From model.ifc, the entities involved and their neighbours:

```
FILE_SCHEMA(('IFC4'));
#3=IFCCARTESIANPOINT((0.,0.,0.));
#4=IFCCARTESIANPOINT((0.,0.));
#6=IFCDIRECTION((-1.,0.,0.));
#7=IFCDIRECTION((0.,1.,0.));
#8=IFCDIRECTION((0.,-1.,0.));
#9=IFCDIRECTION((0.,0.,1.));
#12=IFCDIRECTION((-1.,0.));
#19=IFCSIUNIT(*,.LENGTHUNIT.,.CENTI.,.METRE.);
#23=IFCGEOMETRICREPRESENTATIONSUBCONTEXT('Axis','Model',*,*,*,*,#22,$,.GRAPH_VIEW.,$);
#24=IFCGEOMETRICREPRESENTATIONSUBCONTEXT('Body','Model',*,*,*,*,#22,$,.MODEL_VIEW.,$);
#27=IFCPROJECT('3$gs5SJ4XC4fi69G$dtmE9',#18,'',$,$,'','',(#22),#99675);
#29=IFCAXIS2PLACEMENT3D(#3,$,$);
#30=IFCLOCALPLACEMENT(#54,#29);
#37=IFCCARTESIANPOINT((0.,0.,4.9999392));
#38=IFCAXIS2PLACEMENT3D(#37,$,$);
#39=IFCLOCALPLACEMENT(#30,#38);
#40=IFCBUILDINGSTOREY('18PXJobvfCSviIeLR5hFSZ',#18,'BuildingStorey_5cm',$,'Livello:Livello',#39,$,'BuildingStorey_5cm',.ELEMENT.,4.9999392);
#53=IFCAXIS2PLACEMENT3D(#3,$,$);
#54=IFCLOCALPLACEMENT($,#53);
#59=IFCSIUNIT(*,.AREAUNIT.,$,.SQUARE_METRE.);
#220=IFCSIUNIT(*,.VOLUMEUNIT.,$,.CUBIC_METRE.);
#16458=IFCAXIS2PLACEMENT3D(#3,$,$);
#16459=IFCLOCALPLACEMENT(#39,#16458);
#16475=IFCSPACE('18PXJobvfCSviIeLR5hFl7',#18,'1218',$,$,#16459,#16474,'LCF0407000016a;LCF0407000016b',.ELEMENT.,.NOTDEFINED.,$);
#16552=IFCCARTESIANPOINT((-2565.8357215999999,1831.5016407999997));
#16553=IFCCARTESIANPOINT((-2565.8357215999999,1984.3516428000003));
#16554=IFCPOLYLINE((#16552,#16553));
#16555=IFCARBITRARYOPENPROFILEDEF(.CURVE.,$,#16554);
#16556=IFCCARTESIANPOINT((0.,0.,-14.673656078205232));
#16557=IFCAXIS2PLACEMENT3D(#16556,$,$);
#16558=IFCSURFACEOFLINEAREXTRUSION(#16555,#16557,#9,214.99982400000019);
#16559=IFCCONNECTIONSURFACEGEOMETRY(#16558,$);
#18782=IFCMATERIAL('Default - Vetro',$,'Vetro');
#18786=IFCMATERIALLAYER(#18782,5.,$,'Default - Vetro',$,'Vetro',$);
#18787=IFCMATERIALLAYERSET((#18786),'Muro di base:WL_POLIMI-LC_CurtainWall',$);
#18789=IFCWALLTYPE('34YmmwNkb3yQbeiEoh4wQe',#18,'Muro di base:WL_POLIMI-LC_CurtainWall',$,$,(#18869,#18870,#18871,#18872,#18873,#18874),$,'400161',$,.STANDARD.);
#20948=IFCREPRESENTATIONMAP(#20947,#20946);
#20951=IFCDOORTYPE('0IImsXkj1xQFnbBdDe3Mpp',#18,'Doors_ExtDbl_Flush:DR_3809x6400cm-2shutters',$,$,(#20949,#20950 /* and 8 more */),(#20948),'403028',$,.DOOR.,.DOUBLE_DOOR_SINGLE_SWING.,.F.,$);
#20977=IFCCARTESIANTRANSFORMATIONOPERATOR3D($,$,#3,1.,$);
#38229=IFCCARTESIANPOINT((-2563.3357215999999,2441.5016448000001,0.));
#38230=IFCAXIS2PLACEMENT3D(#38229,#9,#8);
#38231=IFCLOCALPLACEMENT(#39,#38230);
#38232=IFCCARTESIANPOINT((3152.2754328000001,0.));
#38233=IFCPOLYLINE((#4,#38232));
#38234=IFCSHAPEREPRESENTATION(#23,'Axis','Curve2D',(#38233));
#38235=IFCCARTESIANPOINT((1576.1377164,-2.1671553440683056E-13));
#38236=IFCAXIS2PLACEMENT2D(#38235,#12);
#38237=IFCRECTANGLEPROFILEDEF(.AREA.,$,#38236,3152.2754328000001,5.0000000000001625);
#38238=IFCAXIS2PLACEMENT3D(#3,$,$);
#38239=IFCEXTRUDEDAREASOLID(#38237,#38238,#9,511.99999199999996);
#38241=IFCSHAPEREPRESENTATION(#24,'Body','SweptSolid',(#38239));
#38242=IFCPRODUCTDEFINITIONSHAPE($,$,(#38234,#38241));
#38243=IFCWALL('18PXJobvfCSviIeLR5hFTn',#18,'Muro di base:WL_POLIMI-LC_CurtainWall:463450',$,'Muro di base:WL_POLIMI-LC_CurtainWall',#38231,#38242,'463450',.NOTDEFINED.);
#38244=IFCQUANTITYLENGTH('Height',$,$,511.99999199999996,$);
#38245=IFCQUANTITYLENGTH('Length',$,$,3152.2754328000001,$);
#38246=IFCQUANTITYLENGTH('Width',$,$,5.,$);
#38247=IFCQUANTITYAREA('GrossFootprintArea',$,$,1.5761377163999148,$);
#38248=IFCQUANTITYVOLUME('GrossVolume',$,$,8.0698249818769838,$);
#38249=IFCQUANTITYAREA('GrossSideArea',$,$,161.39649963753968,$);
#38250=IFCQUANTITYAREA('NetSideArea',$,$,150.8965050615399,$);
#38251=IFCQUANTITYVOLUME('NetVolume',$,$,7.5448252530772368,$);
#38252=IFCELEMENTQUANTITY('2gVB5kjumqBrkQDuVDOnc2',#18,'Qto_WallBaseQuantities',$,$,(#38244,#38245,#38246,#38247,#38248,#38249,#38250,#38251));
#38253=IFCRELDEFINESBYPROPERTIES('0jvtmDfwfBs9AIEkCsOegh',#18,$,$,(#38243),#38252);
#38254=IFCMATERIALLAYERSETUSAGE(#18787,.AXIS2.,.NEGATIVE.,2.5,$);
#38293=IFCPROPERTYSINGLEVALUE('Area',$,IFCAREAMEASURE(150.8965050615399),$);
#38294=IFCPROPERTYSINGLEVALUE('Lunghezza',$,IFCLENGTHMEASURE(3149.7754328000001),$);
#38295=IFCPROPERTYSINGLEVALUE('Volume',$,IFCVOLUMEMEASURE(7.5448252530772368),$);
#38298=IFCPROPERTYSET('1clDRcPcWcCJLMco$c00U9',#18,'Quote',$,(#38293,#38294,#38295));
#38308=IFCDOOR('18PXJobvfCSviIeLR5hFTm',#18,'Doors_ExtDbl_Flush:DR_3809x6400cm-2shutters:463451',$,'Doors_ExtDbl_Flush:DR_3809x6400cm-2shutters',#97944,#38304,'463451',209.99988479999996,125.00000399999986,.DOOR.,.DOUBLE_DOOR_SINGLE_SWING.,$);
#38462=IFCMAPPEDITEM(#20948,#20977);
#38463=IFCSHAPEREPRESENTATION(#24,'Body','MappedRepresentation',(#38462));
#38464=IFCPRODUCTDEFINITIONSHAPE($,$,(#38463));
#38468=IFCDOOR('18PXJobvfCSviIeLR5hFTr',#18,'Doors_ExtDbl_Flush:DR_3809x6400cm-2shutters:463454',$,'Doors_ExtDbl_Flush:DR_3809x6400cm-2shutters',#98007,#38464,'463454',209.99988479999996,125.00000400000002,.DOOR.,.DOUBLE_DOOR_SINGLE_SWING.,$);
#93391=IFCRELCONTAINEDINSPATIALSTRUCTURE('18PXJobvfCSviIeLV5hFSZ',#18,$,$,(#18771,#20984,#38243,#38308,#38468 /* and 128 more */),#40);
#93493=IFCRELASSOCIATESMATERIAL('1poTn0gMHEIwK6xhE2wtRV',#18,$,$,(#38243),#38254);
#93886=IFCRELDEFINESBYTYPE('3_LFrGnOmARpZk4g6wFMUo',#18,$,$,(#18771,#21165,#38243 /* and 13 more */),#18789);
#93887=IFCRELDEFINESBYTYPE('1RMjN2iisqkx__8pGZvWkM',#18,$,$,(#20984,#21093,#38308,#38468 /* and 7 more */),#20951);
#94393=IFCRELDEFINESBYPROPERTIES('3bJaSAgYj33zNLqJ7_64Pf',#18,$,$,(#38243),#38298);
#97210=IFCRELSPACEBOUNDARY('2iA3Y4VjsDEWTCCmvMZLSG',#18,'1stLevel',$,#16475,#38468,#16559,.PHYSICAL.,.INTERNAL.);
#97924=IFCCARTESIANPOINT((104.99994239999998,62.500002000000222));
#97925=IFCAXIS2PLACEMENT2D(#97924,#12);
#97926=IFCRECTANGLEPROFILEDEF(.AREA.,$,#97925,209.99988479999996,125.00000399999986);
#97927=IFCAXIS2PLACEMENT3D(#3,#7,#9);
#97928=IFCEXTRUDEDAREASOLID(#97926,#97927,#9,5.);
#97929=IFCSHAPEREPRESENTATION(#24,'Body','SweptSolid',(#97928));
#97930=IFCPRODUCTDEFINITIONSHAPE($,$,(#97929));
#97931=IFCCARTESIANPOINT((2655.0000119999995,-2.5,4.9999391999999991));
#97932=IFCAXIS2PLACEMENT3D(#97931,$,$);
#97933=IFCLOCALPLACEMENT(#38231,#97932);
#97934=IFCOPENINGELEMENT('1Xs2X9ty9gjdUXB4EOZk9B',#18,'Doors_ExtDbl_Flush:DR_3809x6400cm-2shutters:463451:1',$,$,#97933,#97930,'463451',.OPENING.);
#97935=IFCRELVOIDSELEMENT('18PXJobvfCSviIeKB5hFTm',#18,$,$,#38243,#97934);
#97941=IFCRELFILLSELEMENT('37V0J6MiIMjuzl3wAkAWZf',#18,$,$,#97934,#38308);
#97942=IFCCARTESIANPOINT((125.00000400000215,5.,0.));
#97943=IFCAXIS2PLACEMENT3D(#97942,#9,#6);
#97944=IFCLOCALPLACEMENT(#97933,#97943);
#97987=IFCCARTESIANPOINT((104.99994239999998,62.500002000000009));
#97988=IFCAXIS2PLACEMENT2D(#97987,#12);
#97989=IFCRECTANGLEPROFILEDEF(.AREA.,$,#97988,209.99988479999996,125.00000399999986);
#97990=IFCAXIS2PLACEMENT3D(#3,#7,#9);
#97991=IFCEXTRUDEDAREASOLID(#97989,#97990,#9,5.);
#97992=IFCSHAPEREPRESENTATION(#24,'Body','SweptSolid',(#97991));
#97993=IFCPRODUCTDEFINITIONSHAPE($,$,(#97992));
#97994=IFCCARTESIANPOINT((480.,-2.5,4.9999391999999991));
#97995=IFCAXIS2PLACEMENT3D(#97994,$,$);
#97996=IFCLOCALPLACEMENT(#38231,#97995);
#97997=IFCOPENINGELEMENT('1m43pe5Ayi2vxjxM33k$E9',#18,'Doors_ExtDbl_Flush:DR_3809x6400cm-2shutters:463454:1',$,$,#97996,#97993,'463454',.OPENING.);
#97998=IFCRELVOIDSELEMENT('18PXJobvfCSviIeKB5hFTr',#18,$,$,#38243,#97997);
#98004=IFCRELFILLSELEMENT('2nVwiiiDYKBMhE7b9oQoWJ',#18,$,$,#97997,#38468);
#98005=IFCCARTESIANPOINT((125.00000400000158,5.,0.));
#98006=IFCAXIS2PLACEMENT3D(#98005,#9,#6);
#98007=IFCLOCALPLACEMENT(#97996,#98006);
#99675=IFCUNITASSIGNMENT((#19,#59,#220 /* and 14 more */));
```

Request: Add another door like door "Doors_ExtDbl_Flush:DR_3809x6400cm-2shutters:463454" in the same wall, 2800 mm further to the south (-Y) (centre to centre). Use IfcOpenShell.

```python
import numpy as np
import ifcopenshell
import ifcopenshell.api.feature
import ifcopenshell.api.geometry
import ifcopenshell.api.pset
import ifcopenshell.api.root
import ifcopenshell.geom
import ifcopenshell.util.element
import ifcopenshell.util.placement
import ifcopenshell.util.shape
import ifcopenshell.util.unit

model = ifcopenshell.open("model.ifc")
unit_scale = ifcopenshell.util.unit.calculate_unit_scale(model)
area_scale = ifcopenshell.util.unit.calculate_unit_scale(model, "AREAUNIT")
volume_scale = ifcopenshell.util.unit.calculate_unit_scale(model, "VOLUMEUNIT")
settings = ifcopenshell.geom.settings()


def volume(element):
    """Net volume in cubic metres, openings subtracted."""
    shape = ifcopenshell.geom.create_shape(settings, element)
    return ifcopenshell.util.shape.get_volume(shape.geometry)


def reuse_history(source, copy):
    """copy_class also copies each property set's owner history, people and application; keep the originals."""
    for rel in copy.IsDefinedBy:
        if rel.is_a("IfcRelDefinesByProperties") and (history := rel.RelatingPropertyDefinition.OwnerHistory):
            rel.RelatingPropertyDefinition.OwnerHistory = source.OwnerHistory
            ifcopenshell.util.element.remove_deep2(model, history)


door = model.by_guid("18PXJobvfCSviIeLR5hFTr")
opening = door.FillsVoids[0].RelatingOpeningElement
wall = opening.VoidsElements[0].RelatingBuildingElement
before = volume(wall)
shift = ifcopenshell.util.placement.get_local_placement(wall.ObjectPlacement)[:3, 0] * 2.8 / unit_scale

# copy_class copies the void relationship, type, container and properties, but no geometry.
new_opening = ifcopenshell.api.root.copy_class(model, product=opening)
new_opening.Representation = ifcopenshell.util.element.copy_deep(
    model, opening.Representation, exclude=["IfcGeometricRepresentationContext", "IfcRepresentationMap"]
)
new_opening.Name = "Doors_ExtDbl_Flush:DR_3809x6400cm-2shutters"
new_opening.Tag = None
reuse_history(opening, new_opening)
new_door = ifcopenshell.api.root.copy_class(model, product=door)
new_door.Representation = ifcopenshell.util.element.copy_deep(
    model, door.Representation, exclude=["IfcGeometricRepresentationContext", "IfcRepresentationMap"]
)
new_door.Name = "Doors_ExtDbl_Flush:DR_3809x6400cm-2shutters"
new_door.Tag = None
reuse_history(door, new_door)
ifcopenshell.api.feature.add_filling(model, opening=new_opening, element=new_door)

for old, new in ((opening, new_opening), (door, new_door)):
    matrix = ifcopenshell.util.placement.get_local_placement(old.ObjectPlacement)
    matrix[:3, 3] += shift
    ifcopenshell.api.geometry.edit_object_placement(model, product=new, matrix=matrix, is_si=False)

# The copied space boundaries still share their surfaces with the original.
for rel in new_door.ProvidesBoundaries:
    if rel.ConnectionGeometry:
        rel.ConnectionGeometry = ifcopenshell.util.element.copy_deep(model, rel.ConnectionGeometry)

# Space boundary surfaces are stored in each space's coordinates; move them too.
for rel in new_door.ProvidesBoundaries:
    if not rel.ConnectionGeometry:
        continue
    surface = rel.ConnectionGeometry.SurfaceOnRelatingElement
    space_matrix = ifcopenshell.util.placement.get_local_placement(rel.RelatingSpace.ObjectPlacement)
    point = np.array(surface.Position.Location.Coordinates) + space_matrix[:3, :3].T @ shift
    surface.Position = model.createIfcAxis2Placement3D(
        model.createIfcCartesianPoint(point.tolist()), surface.Position.Axis, surface.Position.RefDirection
    )

after = volume(wall)
thickness = 0.05  # wall thickness in metres

# Update the wall's stored quantities.
qto = model.by_id(ifcopenshell.util.element.get_pset(wall, "Qto_WallBaseQuantities", should_inherit=False)["id"])
ifcopenshell.api.pset.edit_qto(model, qto=qto, properties={
    "NetSideArea": after / thickness / area_scale,
    "NetVolume": after / volume_scale,
})
pset = model.by_id(ifcopenshell.util.element.get_pset(wall, "Quote", should_inherit=False)["id"])
ifcopenshell.api.pset.edit_pset(model, pset=pset, properties={
    "Area": model.create_entity("IfcAreaMeasure", after / thickness / area_scale),
    "Volume": model.create_entity("IfcVolumeMeasure", after / volume_scale),
})

print(f"wall volume {before:.3f} -> {after:.3f} m3")

model.write("model_updated.ifc")
```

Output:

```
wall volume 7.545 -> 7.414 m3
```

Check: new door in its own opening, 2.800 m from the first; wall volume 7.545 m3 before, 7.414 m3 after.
